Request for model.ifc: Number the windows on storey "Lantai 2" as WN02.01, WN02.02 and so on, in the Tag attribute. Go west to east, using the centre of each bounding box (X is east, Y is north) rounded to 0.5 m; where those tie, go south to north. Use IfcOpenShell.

First a look at what the model holds.

```python
import ifcopenshell
import ifcopenshell.util.element
import ifcopenshell.util.placement

model = ifcopenshell.open("model.ifc")
print(model.schema)
storey = next(s for s in model.by_type("IfcBuildingStorey") if s.Name == "Lantai 2")
windows = [e for e in ifcopenshell.util.element.get_decomposition(storey) if e.is_a("IfcWindow")]
for e in sorted(windows, key=lambda e: e.id()):
    origin = ifcopenshell.util.placement.get_local_placement(e.ObjectPlacement)[:3, 3]
    print(e.id(), e.Tag, e.Name, origin.round(2) + 0.0, sep=" | ")
```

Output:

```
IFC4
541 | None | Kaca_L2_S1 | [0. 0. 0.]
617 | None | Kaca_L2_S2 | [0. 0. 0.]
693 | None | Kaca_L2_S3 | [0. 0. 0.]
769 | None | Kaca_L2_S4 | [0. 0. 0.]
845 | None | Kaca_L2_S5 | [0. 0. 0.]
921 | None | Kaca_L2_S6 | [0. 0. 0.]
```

```python
import ifcopenshell
import ifcopenshell.geom
import ifcopenshell.util.element
import ifcopenshell.util.shape

model = ifcopenshell.open("model.ifc")
settings = ifcopenshell.geom.settings()
settings.set("use-world-coords", True)


def centre(element):
    shape = ifcopenshell.geom.create_shape(settings, element)
    return ifcopenshell.util.shape.get_bbox_centroid(shape.geometry)


storey = next(s for s in model.by_type("IfcBuildingStorey") if s.Name == "Lantai 2")
windows = [e for e in ifcopenshell.util.element.get_decomposition(storey) if e.is_a("IfcWindow")]

# Insertion points can sit at a corner or the storey origin, so sort by the geometry (in metres).
centres = {e: centre(e) for e in windows}
windows.sort(key=lambda e: (round(centres[e][0] / 0.5), centres[e][1]))

for i, e in enumerate(windows, start=1):
    number = f"WN02.{i:02d}"
    e.Tag = number
    print(e.id(), number)

model.write("model_updated.ifc")
```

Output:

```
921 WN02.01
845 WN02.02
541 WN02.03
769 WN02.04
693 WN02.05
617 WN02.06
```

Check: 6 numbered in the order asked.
